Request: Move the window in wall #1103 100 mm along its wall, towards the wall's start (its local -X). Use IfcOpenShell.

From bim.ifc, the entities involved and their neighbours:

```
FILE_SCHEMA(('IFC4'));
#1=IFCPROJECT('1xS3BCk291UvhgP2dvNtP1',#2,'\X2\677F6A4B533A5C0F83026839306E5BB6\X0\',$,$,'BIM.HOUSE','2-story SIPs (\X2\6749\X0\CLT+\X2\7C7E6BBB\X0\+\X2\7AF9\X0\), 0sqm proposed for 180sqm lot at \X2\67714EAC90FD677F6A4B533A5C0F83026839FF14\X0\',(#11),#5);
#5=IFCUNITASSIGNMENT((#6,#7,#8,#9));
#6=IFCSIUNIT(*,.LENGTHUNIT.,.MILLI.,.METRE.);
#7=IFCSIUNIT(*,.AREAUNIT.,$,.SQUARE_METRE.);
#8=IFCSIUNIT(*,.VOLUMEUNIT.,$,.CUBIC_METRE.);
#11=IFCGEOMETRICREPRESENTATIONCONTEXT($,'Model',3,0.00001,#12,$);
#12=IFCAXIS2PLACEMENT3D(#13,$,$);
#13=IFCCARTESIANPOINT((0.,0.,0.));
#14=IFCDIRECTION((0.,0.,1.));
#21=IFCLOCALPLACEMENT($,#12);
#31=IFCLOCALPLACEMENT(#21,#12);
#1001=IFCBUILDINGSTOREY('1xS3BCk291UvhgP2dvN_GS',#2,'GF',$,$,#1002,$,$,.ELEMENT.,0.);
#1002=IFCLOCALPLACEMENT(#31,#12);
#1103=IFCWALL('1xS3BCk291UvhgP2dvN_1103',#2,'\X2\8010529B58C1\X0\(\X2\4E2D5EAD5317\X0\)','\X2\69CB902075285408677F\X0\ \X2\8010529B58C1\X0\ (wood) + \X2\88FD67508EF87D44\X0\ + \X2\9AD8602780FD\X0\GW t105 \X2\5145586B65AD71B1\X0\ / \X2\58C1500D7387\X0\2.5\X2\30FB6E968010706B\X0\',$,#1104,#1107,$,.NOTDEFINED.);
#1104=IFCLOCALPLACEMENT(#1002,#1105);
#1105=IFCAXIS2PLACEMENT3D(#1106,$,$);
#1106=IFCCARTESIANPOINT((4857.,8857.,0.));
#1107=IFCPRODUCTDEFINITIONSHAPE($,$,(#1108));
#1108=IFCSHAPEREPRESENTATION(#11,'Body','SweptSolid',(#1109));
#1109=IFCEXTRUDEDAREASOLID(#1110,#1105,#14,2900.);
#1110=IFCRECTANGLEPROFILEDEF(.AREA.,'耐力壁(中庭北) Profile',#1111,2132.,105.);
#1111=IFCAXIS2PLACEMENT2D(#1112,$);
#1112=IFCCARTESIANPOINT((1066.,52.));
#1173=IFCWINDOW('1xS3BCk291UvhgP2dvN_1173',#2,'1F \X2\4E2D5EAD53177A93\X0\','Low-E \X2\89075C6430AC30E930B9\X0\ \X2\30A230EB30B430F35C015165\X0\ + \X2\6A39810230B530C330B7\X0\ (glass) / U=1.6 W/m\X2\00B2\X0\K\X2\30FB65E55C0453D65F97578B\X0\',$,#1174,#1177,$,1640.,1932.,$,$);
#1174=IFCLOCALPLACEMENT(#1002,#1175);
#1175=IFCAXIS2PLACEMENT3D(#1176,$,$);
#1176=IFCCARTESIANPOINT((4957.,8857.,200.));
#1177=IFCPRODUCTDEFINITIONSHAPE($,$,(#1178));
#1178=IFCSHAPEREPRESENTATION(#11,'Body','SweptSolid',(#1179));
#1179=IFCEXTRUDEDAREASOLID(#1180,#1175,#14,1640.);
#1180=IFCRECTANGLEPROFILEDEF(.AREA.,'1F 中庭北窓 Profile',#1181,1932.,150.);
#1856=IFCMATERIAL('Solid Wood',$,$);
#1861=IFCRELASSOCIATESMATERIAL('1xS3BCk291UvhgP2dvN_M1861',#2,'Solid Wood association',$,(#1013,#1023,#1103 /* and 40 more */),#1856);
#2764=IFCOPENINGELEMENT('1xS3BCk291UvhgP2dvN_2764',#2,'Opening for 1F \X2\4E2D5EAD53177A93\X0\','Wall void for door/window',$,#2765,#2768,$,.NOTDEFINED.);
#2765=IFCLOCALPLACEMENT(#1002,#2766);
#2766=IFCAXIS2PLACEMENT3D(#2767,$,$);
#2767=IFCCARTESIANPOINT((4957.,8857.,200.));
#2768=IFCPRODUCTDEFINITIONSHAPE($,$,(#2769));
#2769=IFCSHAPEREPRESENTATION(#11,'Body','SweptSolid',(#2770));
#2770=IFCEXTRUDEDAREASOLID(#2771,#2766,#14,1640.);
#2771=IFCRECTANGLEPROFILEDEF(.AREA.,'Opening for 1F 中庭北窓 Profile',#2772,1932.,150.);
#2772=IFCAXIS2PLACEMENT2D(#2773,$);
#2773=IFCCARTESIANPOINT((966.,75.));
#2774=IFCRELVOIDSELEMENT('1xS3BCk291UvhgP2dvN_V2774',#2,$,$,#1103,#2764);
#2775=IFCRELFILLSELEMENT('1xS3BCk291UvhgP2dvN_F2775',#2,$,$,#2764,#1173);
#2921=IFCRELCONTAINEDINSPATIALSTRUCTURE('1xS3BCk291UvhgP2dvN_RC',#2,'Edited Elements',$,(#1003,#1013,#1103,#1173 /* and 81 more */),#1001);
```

```python
import ifcopenshell
import ifcopenshell.api.geometry
import ifcopenshell.util.placement

model = ifcopenshell.open("bim.ifc")

window = model.by_guid("1xS3BCk291UvhgP2dvN_1173")
opening = window.FillsVoids[0].RelatingOpeningElement
wall = opening.VoidsElements[0].RelatingBuildingElement

wall_matrix = ifcopenshell.util.placement.get_local_placement(wall.ObjectPlacement)
shift = wall_matrix[:3, 0] * -100.0
before = ifcopenshell.util.placement.get_local_placement(window.ObjectPlacement)[:3, 3].copy()

# The window is not placed relative to its opening, so move both.
for product in (opening, window):
    matrix = ifcopenshell.util.placement.get_local_placement(product.ObjectPlacement)
    matrix[:3, 3] += shift
    ifcopenshell.api.geometry.edit_object_placement(model, product=product, matrix=matrix, is_si=False)

after = ifcopenshell.util.placement.get_local_placement(window.ObjectPlacement)[:3, 3]
print("window moved by", (after - before).round(3) + 0.0)

model.write("bim_v2.ifc")
```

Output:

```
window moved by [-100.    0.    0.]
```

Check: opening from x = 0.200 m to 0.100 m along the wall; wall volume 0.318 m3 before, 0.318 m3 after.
